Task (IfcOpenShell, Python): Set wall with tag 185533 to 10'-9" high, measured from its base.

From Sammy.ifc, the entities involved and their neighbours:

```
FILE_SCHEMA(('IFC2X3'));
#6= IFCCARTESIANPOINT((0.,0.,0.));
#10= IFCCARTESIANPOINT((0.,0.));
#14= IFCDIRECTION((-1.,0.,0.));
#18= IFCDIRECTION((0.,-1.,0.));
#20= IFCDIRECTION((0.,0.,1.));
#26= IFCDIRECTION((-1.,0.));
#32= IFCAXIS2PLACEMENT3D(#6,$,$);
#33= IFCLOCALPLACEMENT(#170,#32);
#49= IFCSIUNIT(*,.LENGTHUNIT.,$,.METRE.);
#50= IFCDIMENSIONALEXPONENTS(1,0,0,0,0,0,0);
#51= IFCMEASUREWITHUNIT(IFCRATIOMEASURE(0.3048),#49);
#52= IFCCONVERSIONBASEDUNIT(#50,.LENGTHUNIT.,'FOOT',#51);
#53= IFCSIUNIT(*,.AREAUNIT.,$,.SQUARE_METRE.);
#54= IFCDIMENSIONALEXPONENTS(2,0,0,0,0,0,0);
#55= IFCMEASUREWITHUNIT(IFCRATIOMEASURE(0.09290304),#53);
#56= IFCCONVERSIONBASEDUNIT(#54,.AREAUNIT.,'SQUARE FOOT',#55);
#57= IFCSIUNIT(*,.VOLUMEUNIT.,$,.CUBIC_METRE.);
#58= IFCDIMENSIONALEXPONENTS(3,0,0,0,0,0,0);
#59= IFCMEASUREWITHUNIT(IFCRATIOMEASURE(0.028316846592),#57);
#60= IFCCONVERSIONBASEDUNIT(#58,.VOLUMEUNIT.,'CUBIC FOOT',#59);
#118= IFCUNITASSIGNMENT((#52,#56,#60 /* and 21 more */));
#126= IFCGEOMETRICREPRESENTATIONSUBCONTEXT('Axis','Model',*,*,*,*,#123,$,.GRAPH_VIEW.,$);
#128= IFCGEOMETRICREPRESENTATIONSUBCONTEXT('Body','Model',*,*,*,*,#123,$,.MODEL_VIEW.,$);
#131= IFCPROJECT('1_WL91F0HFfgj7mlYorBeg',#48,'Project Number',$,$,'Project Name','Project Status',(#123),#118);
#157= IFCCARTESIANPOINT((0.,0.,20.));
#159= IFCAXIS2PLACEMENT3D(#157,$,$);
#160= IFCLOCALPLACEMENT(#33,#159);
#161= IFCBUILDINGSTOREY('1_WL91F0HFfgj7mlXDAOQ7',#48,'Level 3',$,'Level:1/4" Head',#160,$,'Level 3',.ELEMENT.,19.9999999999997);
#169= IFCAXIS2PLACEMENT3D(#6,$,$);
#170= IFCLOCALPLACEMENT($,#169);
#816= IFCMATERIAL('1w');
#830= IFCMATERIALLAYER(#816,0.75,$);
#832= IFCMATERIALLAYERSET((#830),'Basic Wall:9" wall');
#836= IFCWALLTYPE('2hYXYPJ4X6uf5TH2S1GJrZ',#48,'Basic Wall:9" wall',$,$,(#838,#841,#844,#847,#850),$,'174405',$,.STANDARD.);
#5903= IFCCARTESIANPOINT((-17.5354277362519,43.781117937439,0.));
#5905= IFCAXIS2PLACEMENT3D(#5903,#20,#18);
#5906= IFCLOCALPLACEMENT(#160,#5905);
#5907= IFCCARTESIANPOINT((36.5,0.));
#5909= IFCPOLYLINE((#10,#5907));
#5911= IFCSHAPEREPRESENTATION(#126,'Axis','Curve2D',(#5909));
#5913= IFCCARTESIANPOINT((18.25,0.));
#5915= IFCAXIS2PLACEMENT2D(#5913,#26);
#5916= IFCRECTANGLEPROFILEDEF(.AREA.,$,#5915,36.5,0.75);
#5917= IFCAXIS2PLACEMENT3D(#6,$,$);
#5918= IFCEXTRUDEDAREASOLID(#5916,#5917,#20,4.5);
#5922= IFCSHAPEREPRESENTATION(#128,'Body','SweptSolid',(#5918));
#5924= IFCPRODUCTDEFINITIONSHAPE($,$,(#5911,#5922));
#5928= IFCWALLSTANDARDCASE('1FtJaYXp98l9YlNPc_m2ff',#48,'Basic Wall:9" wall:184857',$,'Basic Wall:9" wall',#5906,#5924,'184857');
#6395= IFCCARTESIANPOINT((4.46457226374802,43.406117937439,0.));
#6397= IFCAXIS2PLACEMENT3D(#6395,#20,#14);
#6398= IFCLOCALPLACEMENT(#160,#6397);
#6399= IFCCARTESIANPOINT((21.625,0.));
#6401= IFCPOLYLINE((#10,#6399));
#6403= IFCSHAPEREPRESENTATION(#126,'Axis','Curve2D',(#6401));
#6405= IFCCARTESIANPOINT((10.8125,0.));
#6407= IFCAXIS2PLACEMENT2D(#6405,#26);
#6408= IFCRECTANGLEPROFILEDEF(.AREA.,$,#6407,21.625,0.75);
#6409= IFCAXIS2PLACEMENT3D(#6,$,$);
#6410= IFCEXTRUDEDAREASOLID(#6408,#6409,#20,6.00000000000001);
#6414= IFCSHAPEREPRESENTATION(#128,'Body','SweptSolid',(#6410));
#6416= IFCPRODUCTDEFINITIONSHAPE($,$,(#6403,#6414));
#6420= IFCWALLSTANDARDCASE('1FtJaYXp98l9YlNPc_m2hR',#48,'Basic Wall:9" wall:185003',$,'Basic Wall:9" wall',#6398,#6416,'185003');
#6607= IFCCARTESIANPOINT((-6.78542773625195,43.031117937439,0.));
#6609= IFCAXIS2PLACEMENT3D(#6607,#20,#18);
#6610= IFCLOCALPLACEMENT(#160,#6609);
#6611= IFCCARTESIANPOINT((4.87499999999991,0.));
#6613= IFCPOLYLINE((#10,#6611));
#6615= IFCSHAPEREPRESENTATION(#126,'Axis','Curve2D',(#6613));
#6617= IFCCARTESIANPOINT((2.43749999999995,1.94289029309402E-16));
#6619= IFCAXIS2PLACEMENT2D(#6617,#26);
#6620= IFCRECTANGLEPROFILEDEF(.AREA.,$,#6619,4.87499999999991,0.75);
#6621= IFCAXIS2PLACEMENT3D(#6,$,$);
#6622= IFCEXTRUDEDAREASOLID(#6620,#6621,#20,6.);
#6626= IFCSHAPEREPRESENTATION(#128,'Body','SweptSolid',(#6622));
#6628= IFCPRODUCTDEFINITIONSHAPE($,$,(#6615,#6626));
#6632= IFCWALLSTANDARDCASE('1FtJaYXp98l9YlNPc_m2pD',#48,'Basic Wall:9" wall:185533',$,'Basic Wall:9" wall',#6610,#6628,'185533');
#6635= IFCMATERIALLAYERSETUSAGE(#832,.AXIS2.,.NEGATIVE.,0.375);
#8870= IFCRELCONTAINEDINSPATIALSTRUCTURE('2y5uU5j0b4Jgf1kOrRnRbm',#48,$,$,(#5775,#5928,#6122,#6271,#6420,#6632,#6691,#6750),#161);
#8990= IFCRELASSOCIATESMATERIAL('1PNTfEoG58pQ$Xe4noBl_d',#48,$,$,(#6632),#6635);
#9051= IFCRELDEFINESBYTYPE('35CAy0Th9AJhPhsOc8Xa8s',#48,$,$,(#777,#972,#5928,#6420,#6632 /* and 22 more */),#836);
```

```python
import ifcopenshell
import ifcopenshell.geom
import ifcopenshell.util.representation
import ifcopenshell.util.shape
import ifcopenshell.util.unit

model = ifcopenshell.open("Sammy.ifc")
unit_scale = ifcopenshell.util.unit.calculate_unit_scale(model)
settings = ifcopenshell.geom.settings()


def volume(element):
    """Net volume in cubic metres, openings subtracted."""
    shape = ifcopenshell.geom.create_shape(settings, element)
    return ifcopenshell.util.shape.get_volume(shape.geometry)


wall = model.by_id(6632)
before = volume(wall)

body = ifcopenshell.util.representation.get_representation(wall, "Model", "Body")
solid = body.Items[0]
old_height = solid.Depth
solid.Depth = 129 * 0.0254 / unit_scale
after = volume(wall)

print(f"height {old_height:g} -> {solid.Depth:g}, volume {before:.3f} -> {after:.3f} m3")

model.write("Sammy_edited.ifc")
```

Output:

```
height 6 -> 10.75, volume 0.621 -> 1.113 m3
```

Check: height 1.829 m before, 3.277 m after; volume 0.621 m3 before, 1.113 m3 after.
